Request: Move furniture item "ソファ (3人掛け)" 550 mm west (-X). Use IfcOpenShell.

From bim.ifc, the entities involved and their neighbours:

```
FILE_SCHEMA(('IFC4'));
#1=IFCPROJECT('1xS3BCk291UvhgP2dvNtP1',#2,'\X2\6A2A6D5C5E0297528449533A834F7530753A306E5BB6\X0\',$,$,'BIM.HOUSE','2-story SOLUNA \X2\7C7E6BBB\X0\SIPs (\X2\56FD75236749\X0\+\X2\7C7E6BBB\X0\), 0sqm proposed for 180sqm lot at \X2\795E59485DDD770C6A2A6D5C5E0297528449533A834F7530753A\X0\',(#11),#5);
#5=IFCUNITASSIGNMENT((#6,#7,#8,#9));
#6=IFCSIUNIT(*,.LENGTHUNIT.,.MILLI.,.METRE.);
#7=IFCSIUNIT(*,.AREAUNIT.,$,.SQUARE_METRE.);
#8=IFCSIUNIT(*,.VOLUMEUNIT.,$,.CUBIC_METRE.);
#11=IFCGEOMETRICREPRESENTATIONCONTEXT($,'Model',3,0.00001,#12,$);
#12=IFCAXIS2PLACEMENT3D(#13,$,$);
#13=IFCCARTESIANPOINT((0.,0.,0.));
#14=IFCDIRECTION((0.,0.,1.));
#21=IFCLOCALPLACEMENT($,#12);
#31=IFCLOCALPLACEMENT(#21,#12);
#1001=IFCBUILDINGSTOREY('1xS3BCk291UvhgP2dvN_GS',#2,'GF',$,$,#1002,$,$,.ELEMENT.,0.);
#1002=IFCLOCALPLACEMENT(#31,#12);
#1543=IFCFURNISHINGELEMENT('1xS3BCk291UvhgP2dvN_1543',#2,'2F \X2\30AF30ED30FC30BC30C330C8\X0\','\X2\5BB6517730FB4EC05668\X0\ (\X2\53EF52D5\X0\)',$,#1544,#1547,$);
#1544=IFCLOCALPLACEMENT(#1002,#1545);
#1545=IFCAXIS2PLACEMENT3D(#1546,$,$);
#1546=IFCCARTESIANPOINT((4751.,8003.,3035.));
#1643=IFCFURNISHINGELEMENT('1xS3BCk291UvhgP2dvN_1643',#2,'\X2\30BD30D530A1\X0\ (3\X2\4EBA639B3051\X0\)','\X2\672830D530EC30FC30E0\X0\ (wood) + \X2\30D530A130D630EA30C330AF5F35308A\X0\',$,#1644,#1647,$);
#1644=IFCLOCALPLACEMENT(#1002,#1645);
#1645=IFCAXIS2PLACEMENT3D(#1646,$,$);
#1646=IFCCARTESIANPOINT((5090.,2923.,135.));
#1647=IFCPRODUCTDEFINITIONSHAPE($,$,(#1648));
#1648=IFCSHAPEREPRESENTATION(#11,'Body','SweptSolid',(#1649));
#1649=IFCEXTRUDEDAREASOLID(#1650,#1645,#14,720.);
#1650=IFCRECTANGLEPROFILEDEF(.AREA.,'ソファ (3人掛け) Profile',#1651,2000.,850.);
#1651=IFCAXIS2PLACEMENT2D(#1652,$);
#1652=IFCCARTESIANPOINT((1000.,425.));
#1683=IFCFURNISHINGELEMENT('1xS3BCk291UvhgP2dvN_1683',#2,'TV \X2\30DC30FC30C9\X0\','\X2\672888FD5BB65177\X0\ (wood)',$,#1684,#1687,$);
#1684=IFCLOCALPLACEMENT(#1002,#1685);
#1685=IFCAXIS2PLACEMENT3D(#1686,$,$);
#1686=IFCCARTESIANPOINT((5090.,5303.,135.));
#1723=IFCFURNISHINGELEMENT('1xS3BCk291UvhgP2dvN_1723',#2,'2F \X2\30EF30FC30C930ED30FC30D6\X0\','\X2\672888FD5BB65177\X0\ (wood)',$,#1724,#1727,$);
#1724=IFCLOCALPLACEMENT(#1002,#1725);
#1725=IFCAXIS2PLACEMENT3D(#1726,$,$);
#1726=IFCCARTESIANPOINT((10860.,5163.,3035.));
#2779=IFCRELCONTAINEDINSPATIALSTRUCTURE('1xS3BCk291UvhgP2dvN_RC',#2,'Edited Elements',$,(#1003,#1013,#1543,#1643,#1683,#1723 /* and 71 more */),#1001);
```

```python
import ifcopenshell
import ifcopenshell.api.geometry
import ifcopenshell.util.placement
import ifcopenshell.util.unit

model = ifcopenshell.open("bim.ifc")
unit_scale = ifcopenshell.util.unit.calculate_unit_scale(model)

item = model.by_guid("1xS3BCk291UvhgP2dvN_1643")
matrix = ifcopenshell.util.placement.get_local_placement(item.ObjectPlacement)
matrix[0, 3] -= 0.55 / unit_scale
ifcopenshell.api.geometry.edit_object_placement(model, product=item, matrix=matrix, is_si=False)

print(ifcopenshell.util.placement.get_local_placement(item.ObjectPlacement).round(3) + 0.0)

model.write("bim_edited.ifc")
```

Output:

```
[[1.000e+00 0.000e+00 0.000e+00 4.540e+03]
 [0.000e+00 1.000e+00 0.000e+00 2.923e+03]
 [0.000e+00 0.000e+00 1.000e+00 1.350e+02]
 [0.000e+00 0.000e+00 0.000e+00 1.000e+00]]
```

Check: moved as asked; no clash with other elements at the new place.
